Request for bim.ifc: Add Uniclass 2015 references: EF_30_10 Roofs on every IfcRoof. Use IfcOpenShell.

First a look at what the model holds.

```python
import ifcopenshell

model = ifcopenshell.open("bim.ifc")
print(model.schema)
print("classifications:", [c.Name for c in model.by_type("IfcClassification")])
for ifc_class in ("IfcDoor", "IfcRoof", "IfcStair", "IfcWall", "IfcWindow"):
    print(ifc_class, len(model.by_type(ifc_class)))
```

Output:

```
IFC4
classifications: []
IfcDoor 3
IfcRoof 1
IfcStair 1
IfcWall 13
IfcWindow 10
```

```python
import ifcopenshell
import ifcopenshell.api.classification

model = ifcopenshell.open("bim.ifc")

system = ifcopenshell.api.classification.add_classification(model, classification="Uniclass 2015")

codes = {
    "IfcRoof": ("EF_30_10", "Roofs"),
}
for ifc_class, (code, name) in codes.items():
    products = model.by_type(ifc_class)
    ifcopenshell.api.classification.add_reference(
        model, products=products, classification=system, identification=code, name=name
    )
    print(code, len(products))

model.write("bim-out.ifc")
```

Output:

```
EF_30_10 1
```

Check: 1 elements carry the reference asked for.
